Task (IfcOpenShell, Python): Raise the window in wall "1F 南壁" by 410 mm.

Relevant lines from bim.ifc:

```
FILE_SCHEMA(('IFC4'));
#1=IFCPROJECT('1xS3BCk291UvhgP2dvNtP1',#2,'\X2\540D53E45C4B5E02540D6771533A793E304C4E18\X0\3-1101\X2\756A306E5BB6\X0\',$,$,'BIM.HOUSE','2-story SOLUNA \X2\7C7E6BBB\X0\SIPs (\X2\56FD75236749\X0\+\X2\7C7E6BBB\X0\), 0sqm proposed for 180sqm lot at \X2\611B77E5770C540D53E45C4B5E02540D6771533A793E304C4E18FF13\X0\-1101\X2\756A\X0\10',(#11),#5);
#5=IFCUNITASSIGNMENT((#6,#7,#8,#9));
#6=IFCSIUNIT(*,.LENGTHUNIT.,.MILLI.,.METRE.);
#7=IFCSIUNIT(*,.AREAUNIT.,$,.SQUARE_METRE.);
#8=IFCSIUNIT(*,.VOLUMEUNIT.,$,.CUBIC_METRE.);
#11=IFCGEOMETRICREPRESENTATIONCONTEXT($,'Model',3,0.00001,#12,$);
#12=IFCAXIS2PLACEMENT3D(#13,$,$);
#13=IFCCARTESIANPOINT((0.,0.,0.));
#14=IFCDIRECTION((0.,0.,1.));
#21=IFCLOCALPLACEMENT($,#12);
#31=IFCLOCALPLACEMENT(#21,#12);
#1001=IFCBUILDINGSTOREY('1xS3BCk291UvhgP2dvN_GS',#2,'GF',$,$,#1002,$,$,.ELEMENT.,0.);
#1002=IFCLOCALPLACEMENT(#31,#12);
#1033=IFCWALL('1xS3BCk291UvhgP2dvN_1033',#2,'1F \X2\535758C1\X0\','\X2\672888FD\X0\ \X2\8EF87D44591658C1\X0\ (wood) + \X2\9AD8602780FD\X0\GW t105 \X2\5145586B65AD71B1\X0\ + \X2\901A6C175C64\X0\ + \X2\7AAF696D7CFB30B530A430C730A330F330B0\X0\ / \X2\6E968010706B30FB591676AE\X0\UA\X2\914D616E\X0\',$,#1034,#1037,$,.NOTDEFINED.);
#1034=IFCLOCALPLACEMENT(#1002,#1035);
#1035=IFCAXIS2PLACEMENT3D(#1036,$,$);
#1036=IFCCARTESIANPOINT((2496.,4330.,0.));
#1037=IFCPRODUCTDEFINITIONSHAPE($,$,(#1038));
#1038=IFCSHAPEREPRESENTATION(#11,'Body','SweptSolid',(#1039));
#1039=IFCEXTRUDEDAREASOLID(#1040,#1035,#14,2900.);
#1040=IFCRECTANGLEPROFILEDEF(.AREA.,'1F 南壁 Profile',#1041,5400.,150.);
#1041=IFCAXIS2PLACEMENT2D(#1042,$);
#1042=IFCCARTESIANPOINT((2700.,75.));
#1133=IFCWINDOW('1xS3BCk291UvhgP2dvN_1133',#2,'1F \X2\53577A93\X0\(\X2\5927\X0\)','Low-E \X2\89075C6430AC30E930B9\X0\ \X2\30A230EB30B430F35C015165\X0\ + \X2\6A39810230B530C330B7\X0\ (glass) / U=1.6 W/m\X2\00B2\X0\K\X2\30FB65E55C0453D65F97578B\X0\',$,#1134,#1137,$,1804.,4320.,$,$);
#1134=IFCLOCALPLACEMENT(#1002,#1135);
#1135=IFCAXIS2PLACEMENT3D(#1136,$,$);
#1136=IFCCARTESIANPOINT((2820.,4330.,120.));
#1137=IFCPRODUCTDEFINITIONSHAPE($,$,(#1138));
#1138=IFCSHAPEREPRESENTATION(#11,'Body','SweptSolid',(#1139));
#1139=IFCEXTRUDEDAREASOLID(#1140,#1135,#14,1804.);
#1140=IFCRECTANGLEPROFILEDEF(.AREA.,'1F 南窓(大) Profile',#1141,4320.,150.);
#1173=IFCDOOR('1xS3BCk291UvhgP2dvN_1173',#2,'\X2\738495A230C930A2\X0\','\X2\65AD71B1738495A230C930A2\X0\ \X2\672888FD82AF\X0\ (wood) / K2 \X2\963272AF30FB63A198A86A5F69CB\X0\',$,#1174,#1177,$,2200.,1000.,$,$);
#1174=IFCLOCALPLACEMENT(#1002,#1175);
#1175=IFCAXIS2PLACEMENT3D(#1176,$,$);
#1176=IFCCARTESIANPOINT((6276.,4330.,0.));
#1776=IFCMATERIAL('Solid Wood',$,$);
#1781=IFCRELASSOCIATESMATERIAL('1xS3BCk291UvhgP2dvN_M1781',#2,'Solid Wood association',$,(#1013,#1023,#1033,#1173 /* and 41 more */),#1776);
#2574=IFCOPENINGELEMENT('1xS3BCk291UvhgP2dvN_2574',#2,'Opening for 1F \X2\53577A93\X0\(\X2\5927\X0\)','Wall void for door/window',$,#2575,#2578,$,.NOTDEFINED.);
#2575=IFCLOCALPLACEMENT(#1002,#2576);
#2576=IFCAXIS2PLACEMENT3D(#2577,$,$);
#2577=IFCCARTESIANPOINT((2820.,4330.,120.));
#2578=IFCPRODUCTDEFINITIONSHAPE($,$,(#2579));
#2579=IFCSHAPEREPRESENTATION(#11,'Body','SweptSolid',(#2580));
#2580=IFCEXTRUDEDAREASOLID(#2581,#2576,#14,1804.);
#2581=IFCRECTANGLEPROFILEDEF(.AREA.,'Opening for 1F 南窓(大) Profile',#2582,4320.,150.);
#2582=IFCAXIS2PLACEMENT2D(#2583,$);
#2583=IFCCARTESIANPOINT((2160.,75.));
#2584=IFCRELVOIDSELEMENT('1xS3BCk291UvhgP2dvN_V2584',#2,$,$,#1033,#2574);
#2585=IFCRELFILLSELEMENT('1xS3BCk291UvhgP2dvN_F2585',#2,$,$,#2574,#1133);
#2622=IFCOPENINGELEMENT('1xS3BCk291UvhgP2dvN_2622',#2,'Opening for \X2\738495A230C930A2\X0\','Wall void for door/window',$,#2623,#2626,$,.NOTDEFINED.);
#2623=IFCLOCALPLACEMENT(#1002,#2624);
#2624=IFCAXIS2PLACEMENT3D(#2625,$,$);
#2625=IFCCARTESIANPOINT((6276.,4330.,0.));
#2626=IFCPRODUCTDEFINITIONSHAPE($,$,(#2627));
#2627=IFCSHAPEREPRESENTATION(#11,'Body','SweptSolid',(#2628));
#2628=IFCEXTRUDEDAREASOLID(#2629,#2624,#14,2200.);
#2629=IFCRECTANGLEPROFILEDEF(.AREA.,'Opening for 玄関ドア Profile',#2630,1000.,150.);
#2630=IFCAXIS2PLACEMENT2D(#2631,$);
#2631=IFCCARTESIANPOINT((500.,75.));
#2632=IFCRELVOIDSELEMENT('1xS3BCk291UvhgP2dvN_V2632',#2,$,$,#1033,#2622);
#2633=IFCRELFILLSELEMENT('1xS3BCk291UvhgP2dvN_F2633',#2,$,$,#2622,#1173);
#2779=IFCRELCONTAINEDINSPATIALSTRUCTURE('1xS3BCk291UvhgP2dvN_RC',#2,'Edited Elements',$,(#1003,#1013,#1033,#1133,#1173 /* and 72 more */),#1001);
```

```python
import numpy as np
import ifcopenshell
import ifcopenshell.api.geometry
import ifcopenshell.util.placement
import ifcopenshell.util.unit

model = ifcopenshell.open("bim.ifc")
unit_scale = ifcopenshell.util.unit.calculate_unit_scale(model)

window = model.by_guid("1xS3BCk291UvhgP2dvN_1133")
opening = window.FillsVoids[0].RelatingOpeningElement
dz = 0.41 / unit_scale

shift = np.array([0.0, 0.0, dz])
# The window is not placed relative to its opening, so move both.
for product in (opening, window):
    matrix = ifcopenshell.util.placement.get_local_placement(product.ObjectPlacement)
    matrix[:3, 3] += shift
    ifcopenshell.api.geometry.edit_object_placement(model, product=product, matrix=matrix, is_si=False)

print(f"moved by {dz * unit_scale:+.3f} m")

model.write("bim_rev.ifc")
```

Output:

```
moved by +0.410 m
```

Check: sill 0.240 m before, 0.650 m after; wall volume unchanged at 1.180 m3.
